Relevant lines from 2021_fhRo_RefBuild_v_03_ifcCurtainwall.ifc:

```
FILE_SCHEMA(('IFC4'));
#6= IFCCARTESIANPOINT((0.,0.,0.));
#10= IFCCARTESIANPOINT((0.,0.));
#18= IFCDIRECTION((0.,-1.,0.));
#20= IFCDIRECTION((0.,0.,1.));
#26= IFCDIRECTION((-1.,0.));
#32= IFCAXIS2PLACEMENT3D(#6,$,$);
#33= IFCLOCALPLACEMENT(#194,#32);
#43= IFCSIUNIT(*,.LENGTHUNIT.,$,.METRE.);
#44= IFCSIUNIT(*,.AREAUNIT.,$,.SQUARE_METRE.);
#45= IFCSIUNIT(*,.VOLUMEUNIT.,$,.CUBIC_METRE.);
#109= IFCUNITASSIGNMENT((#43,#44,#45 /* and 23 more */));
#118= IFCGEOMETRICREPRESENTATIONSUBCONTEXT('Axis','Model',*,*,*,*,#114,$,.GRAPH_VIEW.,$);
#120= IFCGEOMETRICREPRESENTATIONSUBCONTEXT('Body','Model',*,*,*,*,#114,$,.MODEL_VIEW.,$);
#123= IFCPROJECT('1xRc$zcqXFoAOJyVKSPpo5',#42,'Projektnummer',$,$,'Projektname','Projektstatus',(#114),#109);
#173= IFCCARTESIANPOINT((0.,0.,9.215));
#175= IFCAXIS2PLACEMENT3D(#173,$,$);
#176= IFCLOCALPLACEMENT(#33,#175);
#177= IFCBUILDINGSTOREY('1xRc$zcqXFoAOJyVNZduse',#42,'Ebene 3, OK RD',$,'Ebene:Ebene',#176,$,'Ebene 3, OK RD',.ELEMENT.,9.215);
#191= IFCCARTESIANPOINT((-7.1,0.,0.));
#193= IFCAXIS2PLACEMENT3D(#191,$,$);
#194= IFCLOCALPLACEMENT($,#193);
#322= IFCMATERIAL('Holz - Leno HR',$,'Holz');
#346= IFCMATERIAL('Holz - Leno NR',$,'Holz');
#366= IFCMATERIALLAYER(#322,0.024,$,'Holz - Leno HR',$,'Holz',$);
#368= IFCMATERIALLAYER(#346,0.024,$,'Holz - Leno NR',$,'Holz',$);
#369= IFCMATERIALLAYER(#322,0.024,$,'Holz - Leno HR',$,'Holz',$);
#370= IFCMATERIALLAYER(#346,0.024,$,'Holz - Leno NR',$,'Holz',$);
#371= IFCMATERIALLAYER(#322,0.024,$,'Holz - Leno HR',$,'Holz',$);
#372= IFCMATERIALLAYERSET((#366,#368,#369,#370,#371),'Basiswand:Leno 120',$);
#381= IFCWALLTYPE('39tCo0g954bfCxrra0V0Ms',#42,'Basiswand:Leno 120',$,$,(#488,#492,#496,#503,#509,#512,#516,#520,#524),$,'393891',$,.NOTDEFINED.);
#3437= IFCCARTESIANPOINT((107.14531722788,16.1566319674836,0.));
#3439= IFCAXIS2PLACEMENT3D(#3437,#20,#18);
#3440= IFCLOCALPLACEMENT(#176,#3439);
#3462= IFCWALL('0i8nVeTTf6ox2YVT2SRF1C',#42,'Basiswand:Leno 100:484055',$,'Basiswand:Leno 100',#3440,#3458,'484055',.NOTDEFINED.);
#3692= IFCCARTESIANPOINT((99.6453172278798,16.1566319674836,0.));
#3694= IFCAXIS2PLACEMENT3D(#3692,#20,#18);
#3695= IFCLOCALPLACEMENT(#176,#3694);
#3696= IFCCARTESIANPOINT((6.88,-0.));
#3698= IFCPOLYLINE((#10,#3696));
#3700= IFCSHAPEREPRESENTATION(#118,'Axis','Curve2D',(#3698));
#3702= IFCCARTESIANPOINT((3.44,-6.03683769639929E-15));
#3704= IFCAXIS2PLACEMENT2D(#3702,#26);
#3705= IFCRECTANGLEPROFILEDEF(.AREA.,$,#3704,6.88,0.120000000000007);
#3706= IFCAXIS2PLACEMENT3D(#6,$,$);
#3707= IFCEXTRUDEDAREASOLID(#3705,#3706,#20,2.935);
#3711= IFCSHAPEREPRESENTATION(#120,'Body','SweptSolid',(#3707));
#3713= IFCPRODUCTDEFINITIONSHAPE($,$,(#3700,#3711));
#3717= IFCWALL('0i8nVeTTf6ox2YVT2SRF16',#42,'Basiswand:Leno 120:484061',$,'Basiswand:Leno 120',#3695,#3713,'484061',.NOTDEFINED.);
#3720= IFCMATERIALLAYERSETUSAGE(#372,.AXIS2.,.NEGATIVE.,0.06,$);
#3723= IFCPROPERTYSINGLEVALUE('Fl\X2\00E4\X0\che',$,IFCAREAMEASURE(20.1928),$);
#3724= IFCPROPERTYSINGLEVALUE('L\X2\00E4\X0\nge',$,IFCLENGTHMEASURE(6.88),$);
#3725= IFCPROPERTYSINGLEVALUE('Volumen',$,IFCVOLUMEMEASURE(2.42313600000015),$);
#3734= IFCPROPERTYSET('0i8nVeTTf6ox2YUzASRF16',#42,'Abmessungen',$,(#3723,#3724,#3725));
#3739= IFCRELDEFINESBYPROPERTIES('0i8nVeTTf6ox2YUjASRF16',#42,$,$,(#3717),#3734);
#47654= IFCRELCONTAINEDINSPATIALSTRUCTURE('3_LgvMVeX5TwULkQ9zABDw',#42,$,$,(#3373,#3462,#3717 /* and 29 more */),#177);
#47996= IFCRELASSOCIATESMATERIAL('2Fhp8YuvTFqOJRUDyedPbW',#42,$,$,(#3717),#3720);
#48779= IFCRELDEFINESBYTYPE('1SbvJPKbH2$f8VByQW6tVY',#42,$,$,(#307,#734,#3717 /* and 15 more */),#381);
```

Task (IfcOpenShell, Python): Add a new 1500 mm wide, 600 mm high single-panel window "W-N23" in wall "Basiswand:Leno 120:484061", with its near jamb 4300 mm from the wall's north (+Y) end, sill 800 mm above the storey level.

```python
import numpy as np
import ifcopenshell
import ifcopenshell.api.feature
import ifcopenshell.api.geometry
import ifcopenshell.api.pset
import ifcopenshell.api.root
import ifcopenshell.api.spatial
import ifcopenshell.geom
import ifcopenshell.util.element
import ifcopenshell.util.placement
import ifcopenshell.util.representation
import ifcopenshell.util.shape
import ifcopenshell.util.unit

model = ifcopenshell.open("2021_fhRo_RefBuild_v_03_ifcCurtainwall.ifc")
unit_scale = ifcopenshell.util.unit.calculate_unit_scale(model)
area_scale = ifcopenshell.util.unit.calculate_unit_scale(model, "AREAUNIT")
volume_scale = ifcopenshell.util.unit.calculate_unit_scale(model, "VOLUMEUNIT")
settings = ifcopenshell.geom.settings()


def volume(element):
    """Net volume in cubic metres, openings subtracted."""
    shape = ifcopenshell.geom.create_shape(settings, element)
    return ifcopenshell.util.shape.get_volume(shape.geometry)


wall = model.by_id(3717)
storey = ifcopenshell.util.element.get_container(wall, ifc_class="IfcBuildingStorey")
context = ifcopenshell.util.representation.get_context(model, "Model", "Body", "MODEL_VIEW")
before = volume(wall)

width, height, from_end, sill = 1.5, 0.6, 4.3, 0.8  # metres

# The wall runs along its own X axis, and the end named is its -X end.
wall_shape = ifcopenshell.geom.create_shape(settings, wall)
x, y, z = ifcopenshell.util.shape.get_vertices(wall_shape.geometry).T
start = x.min() + from_end
face, thickness = float(y.min()), float(y.max() - y.min())
wall_matrix = ifcopenshell.util.placement.get_local_placement(wall.ObjectPlacement)
level = ifcopenshell.util.placement.get_local_placement(storey.ObjectPlacement)[2, 3]


def in_wall(x, y):
    """Placement at x, y metres in the wall's axes, at sill height."""
    matrix = wall_matrix.copy()
    matrix[:, 3] = wall_matrix @ np.array([x / unit_scale, y / unit_scale, 0.0, 1.0])
    matrix[2, 3] = level + sill / unit_scale
    return matrix


# Opening: a box that overshoots both wall faces by 50 mm.
opening = ifcopenshell.api.root.create_entity(model, ifc_class="IfcOpeningElement", predefined_type="OPENING")
box = ifcopenshell.api.geometry.add_wall_representation(
    model, context=context, length=width, height=height, thickness=thickness + 0.1
)
ifcopenshell.api.geometry.assign_representation(model, product=opening, representation=box)
ifcopenshell.api.geometry.edit_object_placement(model, product=opening, matrix=in_wall(start, face - 0.05), is_si=False)
ifcopenshell.api.feature.add_feature(model, feature=opening, element=wall)

window = ifcopenshell.api.root.create_entity(model, ifc_class="IfcWindow", name="W-N23", predefined_type="WINDOW")
window.OverallWidth, window.OverallHeight = width / unit_scale, height / unit_scale
window.PartitioningType = "SINGLE_PANEL"
body = ifcopenshell.api.geometry.add_window_representation(
    model,
    context=context,
    overall_width=window.OverallWidth,
    overall_height=window.OverallHeight,
    partition_type="SINGLE_PANEL",
)
ifcopenshell.api.geometry.assign_representation(model, product=window, representation=body)
ifcopenshell.api.spatial.assign_container(model, products=[window], relating_structure=storey)
ifcopenshell.api.feature.add_filling(model, opening=opening, element=window)

# Centre the window in the wall's thickness.
ifcopenshell.api.geometry.edit_object_placement(model, product=window, matrix=in_wall(start, face), is_si=False)
window_shape = ifcopenshell.geom.create_shape(settings, window)
depth = ifcopenshell.util.shape.get_vertices(window_shape.geometry)[:, 1]
offset = face + thickness / 2 - (depth.min() + depth.max()) / 2
ifcopenshell.api.geometry.edit_object_placement(model, product=window, matrix=in_wall(start, offset), is_si=False)

after = volume(wall)

# Update the wall's stored quantities.
pset = model.by_id(ifcopenshell.util.element.get_pset(wall, "Abmessungen", should_inherit=False)["id"])
ifcopenshell.api.pset.edit_pset(model, pset=pset, properties={
    "Fläche": model.create_entity("IfcAreaMeasure", after / thickness / area_scale),
    "Volumen": model.create_entity("IfcVolumeMeasure", after / volume_scale),
})

print(f"wall volume {before:.3f} -> {after:.3f} m3")

model.write("2021_fhRo_RefBuild_v_03_ifcCurtainwall_v2.ifc")
```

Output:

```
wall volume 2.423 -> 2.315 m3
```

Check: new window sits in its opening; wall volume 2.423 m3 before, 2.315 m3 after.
